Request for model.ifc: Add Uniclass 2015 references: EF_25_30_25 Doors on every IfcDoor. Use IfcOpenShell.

First a look at what the model holds.

```python
import ifcopenshell

model = ifcopenshell.open("model.ifc")
print(model.schema)
print("classifications:", [c.Name for c in model.by_type("IfcClassification")])
for ifc_class in ("IfcDoor", "IfcRoof", "IfcStair", "IfcWall", "IfcWindow"):
    print(ifc_class, len(model.by_type(ifc_class)))
```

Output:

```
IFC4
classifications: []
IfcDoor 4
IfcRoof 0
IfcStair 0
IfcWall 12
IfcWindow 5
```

```python
import ifcopenshell
import ifcopenshell.api.classification

model = ifcopenshell.open("model.ifc")

system = ifcopenshell.api.classification.add_classification(model, classification="Uniclass 2015")

codes = {
    "IfcDoor": ("EF_25_30_25", "Doors"),
}
for ifc_class, (code, name) in codes.items():
    products = model.by_type(ifc_class)
    ifcopenshell.api.classification.add_reference(
        model, products=products, classification=system, identification=code, name=name
    )
    print(code, len(products))

model.write("model-out.ifc")
```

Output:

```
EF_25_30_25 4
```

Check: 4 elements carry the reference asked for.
